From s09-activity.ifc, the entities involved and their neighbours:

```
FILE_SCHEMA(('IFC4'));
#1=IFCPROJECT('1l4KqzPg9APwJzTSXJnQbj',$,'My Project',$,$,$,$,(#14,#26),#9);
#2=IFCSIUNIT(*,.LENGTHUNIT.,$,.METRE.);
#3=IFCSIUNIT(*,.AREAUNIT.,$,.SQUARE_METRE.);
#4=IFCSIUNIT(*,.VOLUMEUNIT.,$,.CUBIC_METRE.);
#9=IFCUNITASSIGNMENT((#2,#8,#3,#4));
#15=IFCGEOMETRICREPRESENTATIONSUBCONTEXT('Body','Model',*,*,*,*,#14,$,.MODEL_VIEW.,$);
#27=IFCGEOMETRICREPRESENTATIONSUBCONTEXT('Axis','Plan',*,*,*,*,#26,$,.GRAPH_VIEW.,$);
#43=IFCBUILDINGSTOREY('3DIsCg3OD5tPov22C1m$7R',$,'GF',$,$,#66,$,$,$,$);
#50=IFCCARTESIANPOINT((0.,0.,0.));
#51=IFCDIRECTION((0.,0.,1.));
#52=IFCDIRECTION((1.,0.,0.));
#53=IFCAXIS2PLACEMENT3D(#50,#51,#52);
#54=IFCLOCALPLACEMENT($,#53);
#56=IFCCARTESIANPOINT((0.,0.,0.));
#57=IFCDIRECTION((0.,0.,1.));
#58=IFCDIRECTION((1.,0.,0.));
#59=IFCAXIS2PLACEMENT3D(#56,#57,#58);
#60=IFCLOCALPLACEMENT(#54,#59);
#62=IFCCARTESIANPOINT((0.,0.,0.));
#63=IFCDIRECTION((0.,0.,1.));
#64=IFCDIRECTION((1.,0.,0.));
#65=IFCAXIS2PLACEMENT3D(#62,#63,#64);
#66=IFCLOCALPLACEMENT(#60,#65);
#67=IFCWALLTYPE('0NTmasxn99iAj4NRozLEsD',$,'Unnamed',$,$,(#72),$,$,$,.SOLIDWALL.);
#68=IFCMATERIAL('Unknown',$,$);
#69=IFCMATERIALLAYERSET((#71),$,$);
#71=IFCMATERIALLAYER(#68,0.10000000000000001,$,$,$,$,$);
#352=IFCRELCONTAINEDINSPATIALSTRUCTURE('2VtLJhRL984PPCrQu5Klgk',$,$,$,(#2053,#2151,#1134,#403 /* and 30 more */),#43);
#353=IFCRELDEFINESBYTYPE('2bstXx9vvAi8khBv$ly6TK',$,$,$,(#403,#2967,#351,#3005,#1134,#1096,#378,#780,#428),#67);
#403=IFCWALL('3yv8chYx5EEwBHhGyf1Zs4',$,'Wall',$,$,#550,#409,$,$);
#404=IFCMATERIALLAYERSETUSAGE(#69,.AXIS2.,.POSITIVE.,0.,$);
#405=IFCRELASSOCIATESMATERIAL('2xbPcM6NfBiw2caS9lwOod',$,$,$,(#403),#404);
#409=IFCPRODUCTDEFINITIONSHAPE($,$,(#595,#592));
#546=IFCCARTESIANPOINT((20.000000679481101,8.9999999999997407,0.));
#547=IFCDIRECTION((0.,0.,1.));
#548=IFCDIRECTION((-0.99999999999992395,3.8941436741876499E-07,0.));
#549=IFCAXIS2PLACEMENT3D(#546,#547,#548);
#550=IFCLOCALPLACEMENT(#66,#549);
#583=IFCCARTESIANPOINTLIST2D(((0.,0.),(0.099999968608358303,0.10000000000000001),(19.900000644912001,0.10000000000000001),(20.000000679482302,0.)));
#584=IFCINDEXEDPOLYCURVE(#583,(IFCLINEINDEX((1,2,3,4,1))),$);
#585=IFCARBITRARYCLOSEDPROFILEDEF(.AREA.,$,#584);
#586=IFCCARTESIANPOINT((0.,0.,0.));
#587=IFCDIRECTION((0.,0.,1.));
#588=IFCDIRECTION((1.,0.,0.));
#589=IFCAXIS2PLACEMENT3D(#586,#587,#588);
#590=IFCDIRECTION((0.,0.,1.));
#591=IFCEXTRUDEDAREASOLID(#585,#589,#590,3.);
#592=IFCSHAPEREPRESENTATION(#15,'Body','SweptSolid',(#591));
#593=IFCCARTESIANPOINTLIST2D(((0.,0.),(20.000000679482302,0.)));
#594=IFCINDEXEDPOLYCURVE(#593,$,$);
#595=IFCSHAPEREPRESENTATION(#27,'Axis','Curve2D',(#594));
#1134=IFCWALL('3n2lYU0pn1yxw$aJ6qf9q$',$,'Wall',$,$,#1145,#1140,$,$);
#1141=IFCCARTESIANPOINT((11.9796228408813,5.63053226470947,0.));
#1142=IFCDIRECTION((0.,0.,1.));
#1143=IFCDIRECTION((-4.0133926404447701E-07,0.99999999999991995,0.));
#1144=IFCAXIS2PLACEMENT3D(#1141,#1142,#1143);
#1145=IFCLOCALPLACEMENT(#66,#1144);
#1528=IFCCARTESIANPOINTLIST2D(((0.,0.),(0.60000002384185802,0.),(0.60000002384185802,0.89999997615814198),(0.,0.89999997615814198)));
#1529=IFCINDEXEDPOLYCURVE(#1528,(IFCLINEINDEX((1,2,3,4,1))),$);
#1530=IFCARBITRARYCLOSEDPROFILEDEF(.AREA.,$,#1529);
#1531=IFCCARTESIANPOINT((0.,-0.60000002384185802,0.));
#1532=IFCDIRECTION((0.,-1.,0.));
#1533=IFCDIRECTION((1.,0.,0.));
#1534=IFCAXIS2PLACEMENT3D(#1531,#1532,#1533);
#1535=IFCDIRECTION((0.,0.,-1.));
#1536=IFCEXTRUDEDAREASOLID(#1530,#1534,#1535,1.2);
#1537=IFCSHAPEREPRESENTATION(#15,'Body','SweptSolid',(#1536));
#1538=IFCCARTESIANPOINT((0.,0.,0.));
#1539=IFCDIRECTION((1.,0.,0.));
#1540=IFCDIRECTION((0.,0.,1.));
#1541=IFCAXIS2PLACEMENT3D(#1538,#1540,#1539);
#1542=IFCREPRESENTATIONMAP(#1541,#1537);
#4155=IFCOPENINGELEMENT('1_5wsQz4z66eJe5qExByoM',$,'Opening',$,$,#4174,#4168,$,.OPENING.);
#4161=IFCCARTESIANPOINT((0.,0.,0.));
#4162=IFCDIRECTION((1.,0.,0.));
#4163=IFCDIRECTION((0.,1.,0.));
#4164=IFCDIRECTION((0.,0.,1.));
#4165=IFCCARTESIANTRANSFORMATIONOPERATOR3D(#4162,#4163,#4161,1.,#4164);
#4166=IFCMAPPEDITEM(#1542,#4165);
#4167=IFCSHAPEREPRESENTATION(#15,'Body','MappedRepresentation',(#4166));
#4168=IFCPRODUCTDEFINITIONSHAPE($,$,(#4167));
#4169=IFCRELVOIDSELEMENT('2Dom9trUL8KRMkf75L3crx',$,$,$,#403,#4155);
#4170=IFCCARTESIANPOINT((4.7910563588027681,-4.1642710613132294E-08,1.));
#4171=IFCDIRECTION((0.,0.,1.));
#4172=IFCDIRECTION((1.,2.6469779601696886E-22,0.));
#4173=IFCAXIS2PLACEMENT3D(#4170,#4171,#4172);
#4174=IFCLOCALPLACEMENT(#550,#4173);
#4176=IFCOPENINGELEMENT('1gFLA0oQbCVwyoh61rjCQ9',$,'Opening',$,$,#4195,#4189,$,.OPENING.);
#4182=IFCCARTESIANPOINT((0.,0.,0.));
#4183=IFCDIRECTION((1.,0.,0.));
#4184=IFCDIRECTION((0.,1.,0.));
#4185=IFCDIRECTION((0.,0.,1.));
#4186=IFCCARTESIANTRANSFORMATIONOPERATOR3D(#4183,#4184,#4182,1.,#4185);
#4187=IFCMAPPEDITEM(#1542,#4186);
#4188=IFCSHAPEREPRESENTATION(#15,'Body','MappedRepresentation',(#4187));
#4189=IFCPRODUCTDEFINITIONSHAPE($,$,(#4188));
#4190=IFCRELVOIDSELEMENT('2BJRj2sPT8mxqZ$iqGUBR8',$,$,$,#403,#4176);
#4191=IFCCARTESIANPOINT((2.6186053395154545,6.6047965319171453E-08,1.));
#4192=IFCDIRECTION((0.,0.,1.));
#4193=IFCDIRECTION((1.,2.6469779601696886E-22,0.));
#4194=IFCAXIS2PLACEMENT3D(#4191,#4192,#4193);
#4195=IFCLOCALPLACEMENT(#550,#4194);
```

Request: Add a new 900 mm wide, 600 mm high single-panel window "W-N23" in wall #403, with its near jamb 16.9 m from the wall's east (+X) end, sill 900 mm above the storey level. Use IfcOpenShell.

```python
import numpy as np
import ifcopenshell
import ifcopenshell.api.feature
import ifcopenshell.api.geometry
import ifcopenshell.api.root
import ifcopenshell.api.spatial
import ifcopenshell.geom
import ifcopenshell.util.element
import ifcopenshell.util.placement
import ifcopenshell.util.representation
import ifcopenshell.util.shape
import ifcopenshell.util.unit

model = ifcopenshell.open("s09-activity.ifc")
unit_scale = ifcopenshell.util.unit.calculate_unit_scale(model)
settings = ifcopenshell.geom.settings()


def volume(element):
    """Net volume in cubic metres, openings subtracted."""
    shape = ifcopenshell.geom.create_shape(settings, element)
    return ifcopenshell.util.shape.get_volume(shape.geometry)


wall = model.by_guid("3yv8chYx5EEwBHhGyf1Zs4")
storey = ifcopenshell.util.element.get_container(wall, ifc_class="IfcBuildingStorey")
context = ifcopenshell.util.representation.get_context(model, "Model", "Body", "MODEL_VIEW")
before = volume(wall)

width, height, from_end, sill = 0.9, 0.6, 16.9, 0.9  # metres

# The wall runs along its own X axis, and the end named is its -X end.
wall_shape = ifcopenshell.geom.create_shape(settings, wall)
x, y, z = ifcopenshell.util.shape.get_vertices(wall_shape.geometry).T
start = x.min() + from_end
face, thickness = float(y.min()), float(y.max() - y.min())
wall_matrix = ifcopenshell.util.placement.get_local_placement(wall.ObjectPlacement)
level = ifcopenshell.util.placement.get_local_placement(storey.ObjectPlacement)[2, 3]


def in_wall(x, y):
    """Placement at x, y metres in the wall's axes, at sill height."""
    matrix = wall_matrix.copy()
    matrix[:, 3] = wall_matrix @ np.array([x / unit_scale, y / unit_scale, 0.0, 1.0])
    matrix[2, 3] = level + sill / unit_scale
    return matrix


# Opening: a box that overshoots both wall faces by 50 mm.
opening = ifcopenshell.api.root.create_entity(model, ifc_class="IfcOpeningElement", predefined_type="OPENING")
box = ifcopenshell.api.geometry.add_wall_representation(
    model, context=context, length=width, height=height, thickness=thickness + 0.1
)
ifcopenshell.api.geometry.assign_representation(model, product=opening, representation=box)
ifcopenshell.api.geometry.edit_object_placement(model, product=opening, matrix=in_wall(start, face - 0.05), is_si=False)
ifcopenshell.api.feature.add_feature(model, feature=opening, element=wall)

window = ifcopenshell.api.root.create_entity(model, ifc_class="IfcWindow", name="W-N23", predefined_type="WINDOW")
window.OverallWidth, window.OverallHeight = width / unit_scale, height / unit_scale
window.PartitioningType = "SINGLE_PANEL"
body = ifcopenshell.api.geometry.add_window_representation(
    model,
    context=context,
    overall_width=window.OverallWidth,
    overall_height=window.OverallHeight,
    partition_type="SINGLE_PANEL",
)
ifcopenshell.api.geometry.assign_representation(model, product=window, representation=body)
ifcopenshell.api.spatial.assign_container(model, products=[window], relating_structure=storey)
ifcopenshell.api.feature.add_filling(model, opening=opening, element=window)

# Centre the window in the wall's thickness.
ifcopenshell.api.geometry.edit_object_placement(model, product=window, matrix=in_wall(start, face), is_si=False)
window_shape = ifcopenshell.geom.create_shape(settings, window)
depth = ifcopenshell.util.shape.get_vertices(window_shape.geometry)[:, 1]
offset = face + thickness / 2 - (depth.min() + depth.max()) / 2
ifcopenshell.api.geometry.edit_object_placement(model, product=window, matrix=in_wall(start, offset), is_si=False)

after = volume(wall)

print(f"wall volume {before:.3f} -> {after:.3f} m3")

model.write("s09-activity_updated.ifc")
```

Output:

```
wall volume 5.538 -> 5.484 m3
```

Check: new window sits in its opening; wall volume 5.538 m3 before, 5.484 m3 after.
